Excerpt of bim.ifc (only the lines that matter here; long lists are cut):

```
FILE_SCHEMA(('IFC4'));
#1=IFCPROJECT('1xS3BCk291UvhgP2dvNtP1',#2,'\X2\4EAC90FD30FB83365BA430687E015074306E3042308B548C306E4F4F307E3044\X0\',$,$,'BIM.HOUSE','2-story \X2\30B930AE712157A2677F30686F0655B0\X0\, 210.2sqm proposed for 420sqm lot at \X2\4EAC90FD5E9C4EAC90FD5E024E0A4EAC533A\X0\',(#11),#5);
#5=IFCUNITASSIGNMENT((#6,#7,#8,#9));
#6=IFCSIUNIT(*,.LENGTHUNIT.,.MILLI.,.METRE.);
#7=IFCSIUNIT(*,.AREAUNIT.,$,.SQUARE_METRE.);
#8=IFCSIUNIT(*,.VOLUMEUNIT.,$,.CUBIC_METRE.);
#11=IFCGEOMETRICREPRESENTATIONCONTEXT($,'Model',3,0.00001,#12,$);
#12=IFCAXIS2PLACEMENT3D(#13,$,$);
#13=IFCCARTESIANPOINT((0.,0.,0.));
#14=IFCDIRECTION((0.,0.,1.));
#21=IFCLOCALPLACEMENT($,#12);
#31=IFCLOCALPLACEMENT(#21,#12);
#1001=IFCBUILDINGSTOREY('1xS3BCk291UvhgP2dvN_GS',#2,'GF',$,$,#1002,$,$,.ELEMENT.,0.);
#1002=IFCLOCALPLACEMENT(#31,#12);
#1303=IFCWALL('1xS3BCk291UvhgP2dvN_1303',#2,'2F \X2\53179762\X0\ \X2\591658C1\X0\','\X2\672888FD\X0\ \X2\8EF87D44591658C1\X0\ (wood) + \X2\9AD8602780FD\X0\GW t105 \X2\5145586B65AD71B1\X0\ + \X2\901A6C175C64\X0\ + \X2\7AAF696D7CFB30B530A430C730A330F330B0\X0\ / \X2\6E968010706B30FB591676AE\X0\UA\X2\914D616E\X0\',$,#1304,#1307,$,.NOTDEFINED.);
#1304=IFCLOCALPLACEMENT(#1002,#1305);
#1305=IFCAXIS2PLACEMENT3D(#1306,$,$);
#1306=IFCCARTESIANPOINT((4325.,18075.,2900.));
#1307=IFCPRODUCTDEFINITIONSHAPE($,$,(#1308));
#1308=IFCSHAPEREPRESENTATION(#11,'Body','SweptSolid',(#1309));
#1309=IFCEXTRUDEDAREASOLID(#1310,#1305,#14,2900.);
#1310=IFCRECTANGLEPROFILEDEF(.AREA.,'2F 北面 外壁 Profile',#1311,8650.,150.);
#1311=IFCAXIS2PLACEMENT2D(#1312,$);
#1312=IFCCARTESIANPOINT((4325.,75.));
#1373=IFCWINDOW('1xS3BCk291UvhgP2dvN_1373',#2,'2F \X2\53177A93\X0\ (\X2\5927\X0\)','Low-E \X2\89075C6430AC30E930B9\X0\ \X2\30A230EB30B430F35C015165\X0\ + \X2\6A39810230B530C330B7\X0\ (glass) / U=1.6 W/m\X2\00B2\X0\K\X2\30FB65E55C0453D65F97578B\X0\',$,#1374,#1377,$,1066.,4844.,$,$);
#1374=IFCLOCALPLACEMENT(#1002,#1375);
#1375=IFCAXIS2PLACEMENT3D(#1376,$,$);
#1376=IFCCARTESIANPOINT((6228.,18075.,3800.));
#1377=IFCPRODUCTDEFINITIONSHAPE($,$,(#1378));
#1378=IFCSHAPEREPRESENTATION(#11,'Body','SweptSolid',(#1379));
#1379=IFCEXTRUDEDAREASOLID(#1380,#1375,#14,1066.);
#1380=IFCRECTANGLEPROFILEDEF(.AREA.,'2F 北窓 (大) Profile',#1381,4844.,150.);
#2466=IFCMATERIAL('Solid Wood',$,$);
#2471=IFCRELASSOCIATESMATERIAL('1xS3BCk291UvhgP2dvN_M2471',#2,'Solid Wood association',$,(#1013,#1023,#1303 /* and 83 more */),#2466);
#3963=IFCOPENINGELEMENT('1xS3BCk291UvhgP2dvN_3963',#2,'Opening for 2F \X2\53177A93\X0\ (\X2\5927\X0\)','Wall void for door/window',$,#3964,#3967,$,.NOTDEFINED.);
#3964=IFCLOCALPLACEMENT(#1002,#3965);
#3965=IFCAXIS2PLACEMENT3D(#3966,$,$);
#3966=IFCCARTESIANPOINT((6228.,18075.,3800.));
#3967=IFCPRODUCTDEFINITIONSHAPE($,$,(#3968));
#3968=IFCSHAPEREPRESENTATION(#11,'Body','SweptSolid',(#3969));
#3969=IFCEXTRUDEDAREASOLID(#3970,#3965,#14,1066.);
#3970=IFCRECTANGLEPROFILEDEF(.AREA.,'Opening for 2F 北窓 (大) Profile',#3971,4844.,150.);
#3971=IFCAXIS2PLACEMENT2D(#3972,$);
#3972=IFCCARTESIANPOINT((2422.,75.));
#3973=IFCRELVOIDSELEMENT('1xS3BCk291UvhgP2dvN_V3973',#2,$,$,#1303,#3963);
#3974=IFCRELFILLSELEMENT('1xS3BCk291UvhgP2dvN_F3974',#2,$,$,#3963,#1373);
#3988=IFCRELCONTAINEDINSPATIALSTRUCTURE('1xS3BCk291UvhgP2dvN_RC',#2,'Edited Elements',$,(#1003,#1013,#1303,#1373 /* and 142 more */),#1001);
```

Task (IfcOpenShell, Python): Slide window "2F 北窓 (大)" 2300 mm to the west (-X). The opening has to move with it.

```python
import ifcopenshell
import ifcopenshell.api.geometry
import ifcopenshell.util.placement
import ifcopenshell.util.unit

model = ifcopenshell.open("bim.ifc")
unit_scale = ifcopenshell.util.unit.calculate_unit_scale(model)

window = model.by_id(1373)
opening = window.FillsVoids[0].RelatingOpeningElement
wall = opening.VoidsElements[0].RelatingBuildingElement

wall_matrix = ifcopenshell.util.placement.get_local_placement(wall.ObjectPlacement)
shift = wall_matrix[:3, 0] * -2.3 / unit_scale
before = ifcopenshell.util.placement.get_local_placement(window.ObjectPlacement)[:3, 3].copy()

# The window is not placed relative to its opening, so move both.
for product in (opening, window):
    matrix = ifcopenshell.util.placement.get_local_placement(product.ObjectPlacement)
    matrix[:3, 3] += shift
    ifcopenshell.api.geometry.edit_object_placement(model, product=product, matrix=matrix, is_si=False)

after = ifcopenshell.util.placement.get_local_placement(window.ObjectPlacement)[:3, 3]
print("window moved by", (after - before).round(3) + 0.0)

model.write("bim_updated.ifc")
```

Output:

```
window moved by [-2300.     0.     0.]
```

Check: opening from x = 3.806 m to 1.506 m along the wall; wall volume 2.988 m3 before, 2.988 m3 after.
